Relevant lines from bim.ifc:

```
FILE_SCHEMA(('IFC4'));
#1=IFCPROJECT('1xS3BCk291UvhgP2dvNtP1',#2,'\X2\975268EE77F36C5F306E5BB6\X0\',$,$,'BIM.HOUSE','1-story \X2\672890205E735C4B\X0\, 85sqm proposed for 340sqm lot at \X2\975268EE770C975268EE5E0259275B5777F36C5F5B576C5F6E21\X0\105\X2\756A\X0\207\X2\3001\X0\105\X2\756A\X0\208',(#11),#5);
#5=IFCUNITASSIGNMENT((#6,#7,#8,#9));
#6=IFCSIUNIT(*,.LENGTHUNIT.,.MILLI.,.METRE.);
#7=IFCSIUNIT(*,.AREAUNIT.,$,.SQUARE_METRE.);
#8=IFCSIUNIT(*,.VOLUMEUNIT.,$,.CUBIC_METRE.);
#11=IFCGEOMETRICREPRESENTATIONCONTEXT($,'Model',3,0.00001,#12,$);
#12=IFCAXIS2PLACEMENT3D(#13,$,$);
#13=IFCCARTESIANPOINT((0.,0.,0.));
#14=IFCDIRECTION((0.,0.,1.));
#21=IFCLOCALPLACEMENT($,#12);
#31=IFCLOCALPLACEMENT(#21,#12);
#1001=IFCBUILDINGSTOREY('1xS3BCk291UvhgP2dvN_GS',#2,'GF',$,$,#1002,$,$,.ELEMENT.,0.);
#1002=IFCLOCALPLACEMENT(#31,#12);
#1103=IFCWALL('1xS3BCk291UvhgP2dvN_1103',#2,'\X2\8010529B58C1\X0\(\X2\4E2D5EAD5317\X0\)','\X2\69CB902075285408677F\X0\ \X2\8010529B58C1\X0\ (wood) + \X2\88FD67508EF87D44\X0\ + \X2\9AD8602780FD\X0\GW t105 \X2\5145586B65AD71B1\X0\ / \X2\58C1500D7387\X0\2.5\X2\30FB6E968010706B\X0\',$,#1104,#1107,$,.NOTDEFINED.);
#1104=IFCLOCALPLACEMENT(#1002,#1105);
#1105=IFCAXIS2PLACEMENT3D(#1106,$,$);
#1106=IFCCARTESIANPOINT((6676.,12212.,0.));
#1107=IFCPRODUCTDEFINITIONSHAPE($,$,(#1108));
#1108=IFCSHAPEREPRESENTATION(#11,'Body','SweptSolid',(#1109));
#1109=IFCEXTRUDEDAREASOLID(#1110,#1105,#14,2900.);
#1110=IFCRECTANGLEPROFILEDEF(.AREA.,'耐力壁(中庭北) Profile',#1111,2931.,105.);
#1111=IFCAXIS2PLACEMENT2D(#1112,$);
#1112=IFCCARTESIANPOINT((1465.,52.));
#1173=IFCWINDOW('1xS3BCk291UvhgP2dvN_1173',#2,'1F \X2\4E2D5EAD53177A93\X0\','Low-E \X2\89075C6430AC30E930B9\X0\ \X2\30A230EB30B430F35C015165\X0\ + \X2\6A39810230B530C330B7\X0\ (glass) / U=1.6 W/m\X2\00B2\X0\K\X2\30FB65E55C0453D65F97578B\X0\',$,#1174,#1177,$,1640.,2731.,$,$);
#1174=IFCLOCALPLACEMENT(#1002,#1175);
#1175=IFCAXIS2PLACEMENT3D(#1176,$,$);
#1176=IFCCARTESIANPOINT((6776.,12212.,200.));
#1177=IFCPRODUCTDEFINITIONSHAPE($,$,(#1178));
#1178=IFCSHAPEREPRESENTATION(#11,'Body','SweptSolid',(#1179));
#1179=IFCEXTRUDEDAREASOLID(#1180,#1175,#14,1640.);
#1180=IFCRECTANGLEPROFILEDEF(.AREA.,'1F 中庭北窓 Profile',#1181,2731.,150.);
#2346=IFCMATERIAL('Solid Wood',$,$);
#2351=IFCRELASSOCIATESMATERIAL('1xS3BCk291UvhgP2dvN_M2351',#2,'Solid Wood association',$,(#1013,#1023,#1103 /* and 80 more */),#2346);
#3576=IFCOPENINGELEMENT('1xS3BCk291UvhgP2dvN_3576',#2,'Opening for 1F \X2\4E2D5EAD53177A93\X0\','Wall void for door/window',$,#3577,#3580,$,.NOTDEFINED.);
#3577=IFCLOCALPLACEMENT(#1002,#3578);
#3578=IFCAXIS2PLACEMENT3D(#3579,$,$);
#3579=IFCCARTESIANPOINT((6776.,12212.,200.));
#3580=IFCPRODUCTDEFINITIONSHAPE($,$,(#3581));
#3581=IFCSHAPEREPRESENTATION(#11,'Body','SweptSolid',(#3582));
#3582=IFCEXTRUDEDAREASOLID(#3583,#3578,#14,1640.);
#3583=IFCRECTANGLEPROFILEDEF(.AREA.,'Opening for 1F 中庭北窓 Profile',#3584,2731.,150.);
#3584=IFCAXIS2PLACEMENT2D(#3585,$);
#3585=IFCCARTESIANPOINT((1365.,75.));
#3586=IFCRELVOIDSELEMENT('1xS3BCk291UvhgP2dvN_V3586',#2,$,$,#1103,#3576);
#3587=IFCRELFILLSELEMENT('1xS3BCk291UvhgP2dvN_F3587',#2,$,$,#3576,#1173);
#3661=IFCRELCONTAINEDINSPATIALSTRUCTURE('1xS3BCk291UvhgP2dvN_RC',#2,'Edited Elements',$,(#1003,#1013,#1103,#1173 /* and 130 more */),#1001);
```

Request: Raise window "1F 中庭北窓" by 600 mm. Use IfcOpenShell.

```python
import numpy as np
import ifcopenshell
import ifcopenshell.api.geometry
import ifcopenshell.util.placement
import ifcopenshell.util.unit

model = ifcopenshell.open("bim.ifc")
unit_scale = ifcopenshell.util.unit.calculate_unit_scale(model)

window = model.by_id(1173)
opening = window.FillsVoids[0].RelatingOpeningElement
dz = 0.6 / unit_scale

shift = np.array([0.0, 0.0, dz])
# The window is not placed relative to its opening, so move both.
for product in (opening, window):
    matrix = ifcopenshell.util.placement.get_local_placement(product.ObjectPlacement)
    matrix[:3, 3] += shift
    ifcopenshell.api.geometry.edit_object_placement(model, product=product, matrix=matrix, is_si=False)

print(f"moved by {dz * unit_scale:+.3f} m")

model.write("bim_edited.ifc")
```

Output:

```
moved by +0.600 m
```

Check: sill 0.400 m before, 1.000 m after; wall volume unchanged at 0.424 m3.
